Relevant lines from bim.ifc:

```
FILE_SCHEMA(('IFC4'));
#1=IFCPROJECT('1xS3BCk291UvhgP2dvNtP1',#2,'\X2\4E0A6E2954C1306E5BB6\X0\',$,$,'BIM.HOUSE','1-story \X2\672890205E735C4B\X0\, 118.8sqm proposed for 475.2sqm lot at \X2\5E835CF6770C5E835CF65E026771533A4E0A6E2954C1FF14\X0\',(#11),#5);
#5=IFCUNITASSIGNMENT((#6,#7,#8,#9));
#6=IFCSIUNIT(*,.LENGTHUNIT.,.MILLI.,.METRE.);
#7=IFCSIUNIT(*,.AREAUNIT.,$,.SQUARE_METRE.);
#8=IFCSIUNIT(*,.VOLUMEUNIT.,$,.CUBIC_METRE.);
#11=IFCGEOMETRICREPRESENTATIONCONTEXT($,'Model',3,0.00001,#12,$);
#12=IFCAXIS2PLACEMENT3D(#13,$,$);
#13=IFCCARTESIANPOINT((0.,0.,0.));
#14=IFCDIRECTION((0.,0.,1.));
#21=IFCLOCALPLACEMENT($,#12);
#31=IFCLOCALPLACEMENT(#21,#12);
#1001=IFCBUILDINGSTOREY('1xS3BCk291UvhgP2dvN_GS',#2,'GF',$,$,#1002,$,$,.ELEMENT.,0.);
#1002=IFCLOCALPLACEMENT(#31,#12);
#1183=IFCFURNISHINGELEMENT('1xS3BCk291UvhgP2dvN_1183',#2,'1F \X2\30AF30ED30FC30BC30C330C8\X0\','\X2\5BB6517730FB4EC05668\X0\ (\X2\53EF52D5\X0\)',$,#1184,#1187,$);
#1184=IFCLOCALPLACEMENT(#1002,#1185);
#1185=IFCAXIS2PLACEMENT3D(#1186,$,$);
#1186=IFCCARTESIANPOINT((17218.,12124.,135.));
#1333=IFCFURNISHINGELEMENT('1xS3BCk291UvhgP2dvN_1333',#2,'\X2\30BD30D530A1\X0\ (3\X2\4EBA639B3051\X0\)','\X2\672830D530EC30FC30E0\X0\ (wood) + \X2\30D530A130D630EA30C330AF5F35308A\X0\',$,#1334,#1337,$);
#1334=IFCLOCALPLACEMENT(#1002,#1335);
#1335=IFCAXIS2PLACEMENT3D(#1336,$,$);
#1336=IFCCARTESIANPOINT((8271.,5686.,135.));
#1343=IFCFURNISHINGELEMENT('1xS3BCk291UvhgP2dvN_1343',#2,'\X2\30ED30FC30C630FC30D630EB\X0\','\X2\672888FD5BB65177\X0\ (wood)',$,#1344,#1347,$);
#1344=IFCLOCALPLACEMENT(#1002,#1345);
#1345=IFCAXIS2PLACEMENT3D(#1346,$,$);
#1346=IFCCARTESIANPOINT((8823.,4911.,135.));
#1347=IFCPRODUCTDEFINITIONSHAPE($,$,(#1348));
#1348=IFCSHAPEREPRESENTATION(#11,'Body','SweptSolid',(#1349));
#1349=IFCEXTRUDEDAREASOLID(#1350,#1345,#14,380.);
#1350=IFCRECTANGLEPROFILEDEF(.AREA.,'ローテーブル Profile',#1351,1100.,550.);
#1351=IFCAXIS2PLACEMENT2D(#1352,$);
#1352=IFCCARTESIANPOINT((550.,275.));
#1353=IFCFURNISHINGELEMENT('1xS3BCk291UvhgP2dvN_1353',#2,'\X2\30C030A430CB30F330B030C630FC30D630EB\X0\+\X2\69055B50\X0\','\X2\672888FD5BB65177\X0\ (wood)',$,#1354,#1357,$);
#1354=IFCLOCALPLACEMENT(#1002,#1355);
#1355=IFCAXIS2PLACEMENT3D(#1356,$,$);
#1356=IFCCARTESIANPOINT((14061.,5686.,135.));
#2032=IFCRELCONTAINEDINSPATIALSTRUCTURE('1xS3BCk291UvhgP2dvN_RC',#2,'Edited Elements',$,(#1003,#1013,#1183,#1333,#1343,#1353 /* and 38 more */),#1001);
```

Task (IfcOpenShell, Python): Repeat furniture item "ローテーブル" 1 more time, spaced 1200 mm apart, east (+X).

```python
import numpy as np
import ifcopenshell
import ifcopenshell.api.geometry
import ifcopenshell.api.root
import ifcopenshell.util.element
import ifcopenshell.util.placement

model = ifcopenshell.open("bim.ifc")


def reuse_history(source, copy):
    """copy_class also copies each property set's owner history, people and application; keep the originals."""
    for rel in copy.IsDefinedBy:
        if rel.is_a("IfcRelDefinesByProperties") and (history := rel.RelatingPropertyDefinition.OwnerHistory):
            rel.RelatingPropertyDefinition.OwnerHistory = source.OwnerHistory
            ifcopenshell.util.element.remove_deep2(model, history)


source = model.by_guid("1xS3BCk291UvhgP2dvN_1343")
base = ifcopenshell.util.placement.get_local_placement(source.ObjectPlacement)
step = np.array([1.0, 0.0, 0.0]) * 1200.0

for i in range(1, 2):
    copy = ifcopenshell.api.root.copy_class(model, product=source)
    copy.Representation = ifcopenshell.util.element.copy_deep(
        model, source.Representation, exclude=["IfcGeometricRepresentationContext", "IfcRepresentationMap"]
    )
    reuse_history(source, copy)
    matrix = base.copy()
    matrix[:3, 3] += i * step
    print("added at", matrix[:3, 3].round(3) + 0.0)
    ifcopenshell.api.geometry.edit_object_placement(model, product=copy, matrix=matrix, is_si=False)

model.write("bim_v2.ifc")
```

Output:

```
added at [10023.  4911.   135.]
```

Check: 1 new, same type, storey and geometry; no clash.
